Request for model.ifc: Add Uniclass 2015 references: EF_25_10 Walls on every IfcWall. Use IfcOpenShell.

First a look at what the model holds.

```python
import ifcopenshell

model = ifcopenshell.open("model.ifc")
print(model.schema)
print("classifications:", [c.Name for c in model.by_type("IfcClassification")])
for ifc_class in ("IfcDoor", "IfcRoof", "IfcStair", "IfcWall", "IfcWindow"):
    print(ifc_class, len(model.by_type(ifc_class)))
```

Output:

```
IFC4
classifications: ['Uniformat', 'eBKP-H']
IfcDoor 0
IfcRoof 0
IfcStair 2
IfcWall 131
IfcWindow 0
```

```python
import ifcopenshell
import ifcopenshell.api.classification

model = ifcopenshell.open("model.ifc")

system = ifcopenshell.api.classification.add_classification(model, classification="Uniclass 2015")

codes = {
    "IfcWall": ("EF_25_10", "Walls"),
}
for ifc_class, (code, name) in codes.items():
    products = model.by_type(ifc_class)
    ifcopenshell.api.classification.add_reference(
        model, products=products, classification=system, identification=code, name=name
    )
    print(code, len(products))

model.write("model_rev.ifc")
```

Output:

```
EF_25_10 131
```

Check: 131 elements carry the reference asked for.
